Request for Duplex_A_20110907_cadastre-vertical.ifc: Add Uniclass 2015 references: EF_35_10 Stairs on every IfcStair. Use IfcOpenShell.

First a look at what the model holds.

```python
import ifcopenshell

model = ifcopenshell.open("Duplex_A_20110907_cadastre-vertical.ifc")
print(model.schema)
print("classifications:", [c.Name for c in model.by_type("IfcClassification")])
for ifc_class in ("IfcDoor", "IfcRoof", "IfcStair", "IfcWall", "IfcWindow"):
    print(ifc_class, len(model.by_type(ifc_class)))
```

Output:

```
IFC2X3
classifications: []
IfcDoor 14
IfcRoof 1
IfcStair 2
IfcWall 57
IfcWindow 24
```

```python
import ifcopenshell
import ifcopenshell.api.classification

model = ifcopenshell.open("Duplex_A_20110907_cadastre-vertical.ifc")

# IFC2X3 requires Source and Edition and has no link from the project to the system.
system = model.create_entity("IfcClassification", Source="NBS", Edition="2015", Name="Uniclass 2015")

codes = {
    "IfcStair": ("EF_35_10", "Stairs"),
}
for ifc_class, (code, name) in codes.items():
    products = model.by_type(ifc_class)
    ifcopenshell.api.classification.add_reference(
        model, products=products, classification=system, identification=code, name=name
    )
    print(code, len(products))

model.write("Duplex_A_20110907_cadastre-vertical-out.ifc")
```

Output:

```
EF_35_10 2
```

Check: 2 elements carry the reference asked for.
